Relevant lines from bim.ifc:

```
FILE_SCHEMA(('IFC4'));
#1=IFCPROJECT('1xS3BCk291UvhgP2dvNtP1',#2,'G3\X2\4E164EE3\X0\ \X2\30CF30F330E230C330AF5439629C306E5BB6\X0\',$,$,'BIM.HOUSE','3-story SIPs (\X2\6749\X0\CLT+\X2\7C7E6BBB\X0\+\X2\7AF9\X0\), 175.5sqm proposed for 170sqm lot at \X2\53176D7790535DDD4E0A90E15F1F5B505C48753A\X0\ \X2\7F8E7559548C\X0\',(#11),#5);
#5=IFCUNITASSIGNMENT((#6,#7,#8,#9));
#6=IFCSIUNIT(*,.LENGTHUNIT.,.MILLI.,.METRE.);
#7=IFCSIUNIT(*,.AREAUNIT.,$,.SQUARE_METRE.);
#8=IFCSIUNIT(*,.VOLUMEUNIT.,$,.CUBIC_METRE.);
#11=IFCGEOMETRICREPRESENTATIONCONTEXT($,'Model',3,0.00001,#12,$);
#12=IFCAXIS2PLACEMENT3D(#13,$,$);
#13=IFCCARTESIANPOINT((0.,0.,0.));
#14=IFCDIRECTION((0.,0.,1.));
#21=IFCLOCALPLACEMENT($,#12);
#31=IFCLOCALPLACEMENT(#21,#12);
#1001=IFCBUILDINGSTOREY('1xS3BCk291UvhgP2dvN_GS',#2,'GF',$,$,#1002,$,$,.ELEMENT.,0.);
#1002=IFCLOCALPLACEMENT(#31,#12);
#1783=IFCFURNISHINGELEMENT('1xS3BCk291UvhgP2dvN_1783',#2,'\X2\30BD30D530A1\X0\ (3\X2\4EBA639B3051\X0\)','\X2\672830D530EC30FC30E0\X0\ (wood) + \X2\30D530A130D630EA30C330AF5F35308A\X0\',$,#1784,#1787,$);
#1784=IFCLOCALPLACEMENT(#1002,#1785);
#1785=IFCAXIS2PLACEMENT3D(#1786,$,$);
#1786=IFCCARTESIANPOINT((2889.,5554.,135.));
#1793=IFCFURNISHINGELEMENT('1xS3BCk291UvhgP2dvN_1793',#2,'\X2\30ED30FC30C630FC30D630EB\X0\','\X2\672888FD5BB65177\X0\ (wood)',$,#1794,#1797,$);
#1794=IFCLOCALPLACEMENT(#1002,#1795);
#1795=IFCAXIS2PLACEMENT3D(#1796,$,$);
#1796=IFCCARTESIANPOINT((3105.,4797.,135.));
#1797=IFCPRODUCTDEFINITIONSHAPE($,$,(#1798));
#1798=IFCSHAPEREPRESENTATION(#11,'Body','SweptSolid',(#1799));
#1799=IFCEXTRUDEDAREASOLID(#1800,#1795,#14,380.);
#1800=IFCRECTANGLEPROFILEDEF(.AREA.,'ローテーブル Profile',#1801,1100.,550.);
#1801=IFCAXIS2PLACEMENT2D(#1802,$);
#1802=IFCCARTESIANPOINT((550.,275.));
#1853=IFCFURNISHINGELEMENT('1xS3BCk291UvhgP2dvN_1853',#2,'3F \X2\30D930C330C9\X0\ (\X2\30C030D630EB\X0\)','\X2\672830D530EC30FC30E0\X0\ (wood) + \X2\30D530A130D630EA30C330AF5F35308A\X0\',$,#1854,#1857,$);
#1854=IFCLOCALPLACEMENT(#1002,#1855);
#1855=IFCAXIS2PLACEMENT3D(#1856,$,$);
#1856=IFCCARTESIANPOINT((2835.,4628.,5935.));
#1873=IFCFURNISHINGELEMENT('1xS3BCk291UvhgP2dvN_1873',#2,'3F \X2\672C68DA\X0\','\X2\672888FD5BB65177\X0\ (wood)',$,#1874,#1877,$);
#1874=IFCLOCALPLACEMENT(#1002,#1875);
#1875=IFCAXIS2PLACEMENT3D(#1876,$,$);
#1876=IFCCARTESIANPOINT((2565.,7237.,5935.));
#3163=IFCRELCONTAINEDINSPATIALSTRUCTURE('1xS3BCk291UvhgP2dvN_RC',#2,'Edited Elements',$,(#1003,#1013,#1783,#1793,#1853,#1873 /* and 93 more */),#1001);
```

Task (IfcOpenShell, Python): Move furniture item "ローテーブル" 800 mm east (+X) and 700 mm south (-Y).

```python
import ifcopenshell
import ifcopenshell.api.geometry
import ifcopenshell.util.placement
import ifcopenshell.util.unit

model = ifcopenshell.open("bim.ifc")
unit_scale = ifcopenshell.util.unit.calculate_unit_scale(model)

item = model.by_id(1793)
matrix = ifcopenshell.util.placement.get_local_placement(item.ObjectPlacement)
matrix[0, 3] += 0.8 / unit_scale
matrix[1, 3] -= 0.7 / unit_scale
ifcopenshell.api.geometry.edit_object_placement(model, product=item, matrix=matrix, is_si=False)

print(ifcopenshell.util.placement.get_local_placement(item.ObjectPlacement).round(3) + 0.0)

model.write("bim_edited.ifc")
```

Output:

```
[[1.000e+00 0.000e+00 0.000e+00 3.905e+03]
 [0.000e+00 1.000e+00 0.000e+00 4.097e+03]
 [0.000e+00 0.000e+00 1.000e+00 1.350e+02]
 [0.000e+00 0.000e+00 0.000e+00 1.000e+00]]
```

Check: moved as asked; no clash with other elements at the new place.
